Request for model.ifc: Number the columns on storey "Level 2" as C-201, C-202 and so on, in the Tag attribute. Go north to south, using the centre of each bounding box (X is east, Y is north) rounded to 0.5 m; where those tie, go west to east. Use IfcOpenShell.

First a look at what the model holds.

```python
import ifcopenshell
import ifcopenshell.util.element
import ifcopenshell.util.placement

model = ifcopenshell.open("model.ifc")
print(model.schema)
storey = next(s for s in model.by_type("IfcBuildingStorey") if s.Name == "Level 2")
columns = [e for e in ifcopenshell.util.element.get_decomposition(storey) if e.is_a("IfcColumn")]
for e in sorted(columns, key=lambda e: e.id()):
    origin = ifcopenshell.util.placement.get_local_placement(e.ObjectPlacement)[:3, 3]
    print(e.id(), e.Tag, e.Name, origin.round(2) + 0.0, sep=" | ")
```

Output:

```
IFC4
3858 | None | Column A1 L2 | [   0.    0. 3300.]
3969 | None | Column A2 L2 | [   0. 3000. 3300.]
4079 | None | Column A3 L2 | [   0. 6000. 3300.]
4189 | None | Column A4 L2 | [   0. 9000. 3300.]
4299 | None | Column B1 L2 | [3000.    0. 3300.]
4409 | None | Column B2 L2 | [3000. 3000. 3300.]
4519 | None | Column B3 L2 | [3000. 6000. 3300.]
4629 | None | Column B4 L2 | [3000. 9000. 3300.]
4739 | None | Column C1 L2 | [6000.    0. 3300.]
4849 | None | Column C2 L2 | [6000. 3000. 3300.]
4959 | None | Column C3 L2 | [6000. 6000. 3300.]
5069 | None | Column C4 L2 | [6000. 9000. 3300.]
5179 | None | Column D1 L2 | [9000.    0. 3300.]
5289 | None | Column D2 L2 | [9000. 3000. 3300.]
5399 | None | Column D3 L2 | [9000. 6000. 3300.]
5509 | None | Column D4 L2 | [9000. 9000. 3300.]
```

```python
import ifcopenshell
import ifcopenshell.geom
import ifcopenshell.util.element
import ifcopenshell.util.shape

model = ifcopenshell.open("model.ifc")
settings = ifcopenshell.geom.settings()
settings.set("use-world-coords", True)


def centre(element):
    shape = ifcopenshell.geom.create_shape(settings, element)
    return ifcopenshell.util.shape.get_bbox_centroid(shape.geometry)


storey = next(s for s in model.by_type("IfcBuildingStorey") if s.Name == "Level 2")
columns = [e for e in ifcopenshell.util.element.get_decomposition(storey) if e.is_a("IfcColumn")]

# Insertion points can sit at a corner or the storey origin, so sort by the geometry (in metres).
centres = {e: centre(e) for e in columns}
columns.sort(key=lambda e: (-round(centres[e][1] / 0.5), centres[e][0]))

for i, e in enumerate(columns, start=1):
    number = f"C-2{i:02d}"
    e.Tag = number
    print(e.id(), number)

model.write("model-out.ifc")
```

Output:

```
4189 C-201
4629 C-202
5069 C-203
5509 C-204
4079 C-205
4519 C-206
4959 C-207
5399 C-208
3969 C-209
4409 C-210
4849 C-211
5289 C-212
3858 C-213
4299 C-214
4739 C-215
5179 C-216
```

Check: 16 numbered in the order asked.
